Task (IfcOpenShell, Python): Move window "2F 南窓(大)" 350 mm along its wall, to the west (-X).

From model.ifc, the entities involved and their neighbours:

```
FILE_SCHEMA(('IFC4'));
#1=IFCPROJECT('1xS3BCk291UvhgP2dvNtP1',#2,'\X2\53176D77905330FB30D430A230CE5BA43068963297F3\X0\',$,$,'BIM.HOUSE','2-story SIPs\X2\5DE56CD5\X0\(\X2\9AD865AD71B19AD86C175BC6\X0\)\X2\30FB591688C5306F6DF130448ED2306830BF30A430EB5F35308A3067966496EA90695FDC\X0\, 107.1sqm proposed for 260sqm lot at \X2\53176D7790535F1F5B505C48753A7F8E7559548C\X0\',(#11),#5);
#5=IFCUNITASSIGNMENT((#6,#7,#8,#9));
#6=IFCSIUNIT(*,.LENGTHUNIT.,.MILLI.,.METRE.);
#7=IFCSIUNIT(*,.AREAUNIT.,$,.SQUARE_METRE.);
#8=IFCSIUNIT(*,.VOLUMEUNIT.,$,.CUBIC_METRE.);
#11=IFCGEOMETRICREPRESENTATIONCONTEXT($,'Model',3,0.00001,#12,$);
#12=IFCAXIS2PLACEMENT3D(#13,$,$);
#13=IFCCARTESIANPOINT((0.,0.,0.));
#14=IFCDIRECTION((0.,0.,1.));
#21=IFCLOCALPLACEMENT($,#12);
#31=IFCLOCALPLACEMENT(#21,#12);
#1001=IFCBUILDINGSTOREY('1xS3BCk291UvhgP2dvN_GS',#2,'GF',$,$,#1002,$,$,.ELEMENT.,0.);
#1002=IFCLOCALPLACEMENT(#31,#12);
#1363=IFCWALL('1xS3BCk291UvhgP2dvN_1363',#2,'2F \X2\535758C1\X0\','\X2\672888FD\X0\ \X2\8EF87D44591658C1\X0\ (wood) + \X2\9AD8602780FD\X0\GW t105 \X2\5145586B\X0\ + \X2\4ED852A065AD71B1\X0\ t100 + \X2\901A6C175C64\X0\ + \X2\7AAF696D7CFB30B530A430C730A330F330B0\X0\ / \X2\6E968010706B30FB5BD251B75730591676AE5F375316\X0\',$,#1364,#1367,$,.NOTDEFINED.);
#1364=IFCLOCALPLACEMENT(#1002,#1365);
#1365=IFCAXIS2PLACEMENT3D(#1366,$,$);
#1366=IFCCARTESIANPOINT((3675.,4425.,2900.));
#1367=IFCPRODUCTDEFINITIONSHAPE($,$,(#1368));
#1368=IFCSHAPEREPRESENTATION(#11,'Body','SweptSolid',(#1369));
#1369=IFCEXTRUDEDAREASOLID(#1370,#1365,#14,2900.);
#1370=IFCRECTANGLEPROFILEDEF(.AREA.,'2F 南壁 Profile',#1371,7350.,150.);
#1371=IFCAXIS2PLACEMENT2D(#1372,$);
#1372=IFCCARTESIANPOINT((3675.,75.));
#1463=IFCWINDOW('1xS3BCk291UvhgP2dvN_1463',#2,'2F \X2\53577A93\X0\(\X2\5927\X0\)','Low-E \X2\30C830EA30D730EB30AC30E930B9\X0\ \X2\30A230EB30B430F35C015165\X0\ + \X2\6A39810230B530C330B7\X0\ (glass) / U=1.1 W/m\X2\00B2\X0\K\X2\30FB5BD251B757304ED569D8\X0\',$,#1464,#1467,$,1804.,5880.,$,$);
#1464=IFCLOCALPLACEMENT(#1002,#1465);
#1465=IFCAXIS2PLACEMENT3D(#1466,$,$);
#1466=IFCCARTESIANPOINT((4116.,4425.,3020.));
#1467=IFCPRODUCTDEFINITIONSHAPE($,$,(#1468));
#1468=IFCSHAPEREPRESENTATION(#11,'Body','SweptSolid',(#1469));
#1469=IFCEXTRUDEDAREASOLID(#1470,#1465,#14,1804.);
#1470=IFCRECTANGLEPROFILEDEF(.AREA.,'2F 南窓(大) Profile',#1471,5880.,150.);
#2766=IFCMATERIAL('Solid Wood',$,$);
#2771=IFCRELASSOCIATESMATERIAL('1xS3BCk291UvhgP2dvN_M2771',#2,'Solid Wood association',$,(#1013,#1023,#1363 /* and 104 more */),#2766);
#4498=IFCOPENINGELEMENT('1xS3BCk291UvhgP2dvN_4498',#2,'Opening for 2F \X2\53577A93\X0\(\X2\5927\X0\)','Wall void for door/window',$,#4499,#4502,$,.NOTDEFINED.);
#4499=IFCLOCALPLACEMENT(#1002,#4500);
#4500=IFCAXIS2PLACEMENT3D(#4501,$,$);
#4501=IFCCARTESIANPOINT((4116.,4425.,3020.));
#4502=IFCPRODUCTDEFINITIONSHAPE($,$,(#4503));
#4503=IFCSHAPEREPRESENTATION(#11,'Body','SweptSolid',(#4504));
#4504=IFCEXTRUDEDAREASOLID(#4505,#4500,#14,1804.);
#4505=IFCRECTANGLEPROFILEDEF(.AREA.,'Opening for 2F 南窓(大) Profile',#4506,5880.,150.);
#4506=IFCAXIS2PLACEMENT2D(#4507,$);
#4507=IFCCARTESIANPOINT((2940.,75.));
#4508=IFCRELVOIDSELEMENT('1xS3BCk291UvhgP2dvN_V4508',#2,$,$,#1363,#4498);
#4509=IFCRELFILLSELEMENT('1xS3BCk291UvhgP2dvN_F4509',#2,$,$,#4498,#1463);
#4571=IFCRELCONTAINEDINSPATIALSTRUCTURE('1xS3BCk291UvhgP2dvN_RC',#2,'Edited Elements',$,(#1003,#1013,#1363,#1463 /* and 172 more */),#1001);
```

```python
import ifcopenshell
import ifcopenshell.api.geometry
import ifcopenshell.util.placement

model = ifcopenshell.open("model.ifc")

window = model.by_id(1463)
opening = window.FillsVoids[0].RelatingOpeningElement
wall = opening.VoidsElements[0].RelatingBuildingElement

wall_matrix = ifcopenshell.util.placement.get_local_placement(wall.ObjectPlacement)
shift = wall_matrix[:3, 0] * -350.0
before = ifcopenshell.util.placement.get_local_placement(window.ObjectPlacement)[:3, 3].copy()

# The window is not placed relative to its opening, so move both.
for product in (opening, window):
    matrix = ifcopenshell.util.placement.get_local_placement(product.ObjectPlacement)
    matrix[:3, 3] += shift
    ifcopenshell.api.geometry.edit_object_placement(model, product=product, matrix=matrix, is_si=False)

after = ifcopenshell.util.placement.get_local_placement(window.ObjectPlacement)[:3, 3]
print("window moved by", (after - before).round(3) + 0.0)

model.write("model_v2.ifc")
```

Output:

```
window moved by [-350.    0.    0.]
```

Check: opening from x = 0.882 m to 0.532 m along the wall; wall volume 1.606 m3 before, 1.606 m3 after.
